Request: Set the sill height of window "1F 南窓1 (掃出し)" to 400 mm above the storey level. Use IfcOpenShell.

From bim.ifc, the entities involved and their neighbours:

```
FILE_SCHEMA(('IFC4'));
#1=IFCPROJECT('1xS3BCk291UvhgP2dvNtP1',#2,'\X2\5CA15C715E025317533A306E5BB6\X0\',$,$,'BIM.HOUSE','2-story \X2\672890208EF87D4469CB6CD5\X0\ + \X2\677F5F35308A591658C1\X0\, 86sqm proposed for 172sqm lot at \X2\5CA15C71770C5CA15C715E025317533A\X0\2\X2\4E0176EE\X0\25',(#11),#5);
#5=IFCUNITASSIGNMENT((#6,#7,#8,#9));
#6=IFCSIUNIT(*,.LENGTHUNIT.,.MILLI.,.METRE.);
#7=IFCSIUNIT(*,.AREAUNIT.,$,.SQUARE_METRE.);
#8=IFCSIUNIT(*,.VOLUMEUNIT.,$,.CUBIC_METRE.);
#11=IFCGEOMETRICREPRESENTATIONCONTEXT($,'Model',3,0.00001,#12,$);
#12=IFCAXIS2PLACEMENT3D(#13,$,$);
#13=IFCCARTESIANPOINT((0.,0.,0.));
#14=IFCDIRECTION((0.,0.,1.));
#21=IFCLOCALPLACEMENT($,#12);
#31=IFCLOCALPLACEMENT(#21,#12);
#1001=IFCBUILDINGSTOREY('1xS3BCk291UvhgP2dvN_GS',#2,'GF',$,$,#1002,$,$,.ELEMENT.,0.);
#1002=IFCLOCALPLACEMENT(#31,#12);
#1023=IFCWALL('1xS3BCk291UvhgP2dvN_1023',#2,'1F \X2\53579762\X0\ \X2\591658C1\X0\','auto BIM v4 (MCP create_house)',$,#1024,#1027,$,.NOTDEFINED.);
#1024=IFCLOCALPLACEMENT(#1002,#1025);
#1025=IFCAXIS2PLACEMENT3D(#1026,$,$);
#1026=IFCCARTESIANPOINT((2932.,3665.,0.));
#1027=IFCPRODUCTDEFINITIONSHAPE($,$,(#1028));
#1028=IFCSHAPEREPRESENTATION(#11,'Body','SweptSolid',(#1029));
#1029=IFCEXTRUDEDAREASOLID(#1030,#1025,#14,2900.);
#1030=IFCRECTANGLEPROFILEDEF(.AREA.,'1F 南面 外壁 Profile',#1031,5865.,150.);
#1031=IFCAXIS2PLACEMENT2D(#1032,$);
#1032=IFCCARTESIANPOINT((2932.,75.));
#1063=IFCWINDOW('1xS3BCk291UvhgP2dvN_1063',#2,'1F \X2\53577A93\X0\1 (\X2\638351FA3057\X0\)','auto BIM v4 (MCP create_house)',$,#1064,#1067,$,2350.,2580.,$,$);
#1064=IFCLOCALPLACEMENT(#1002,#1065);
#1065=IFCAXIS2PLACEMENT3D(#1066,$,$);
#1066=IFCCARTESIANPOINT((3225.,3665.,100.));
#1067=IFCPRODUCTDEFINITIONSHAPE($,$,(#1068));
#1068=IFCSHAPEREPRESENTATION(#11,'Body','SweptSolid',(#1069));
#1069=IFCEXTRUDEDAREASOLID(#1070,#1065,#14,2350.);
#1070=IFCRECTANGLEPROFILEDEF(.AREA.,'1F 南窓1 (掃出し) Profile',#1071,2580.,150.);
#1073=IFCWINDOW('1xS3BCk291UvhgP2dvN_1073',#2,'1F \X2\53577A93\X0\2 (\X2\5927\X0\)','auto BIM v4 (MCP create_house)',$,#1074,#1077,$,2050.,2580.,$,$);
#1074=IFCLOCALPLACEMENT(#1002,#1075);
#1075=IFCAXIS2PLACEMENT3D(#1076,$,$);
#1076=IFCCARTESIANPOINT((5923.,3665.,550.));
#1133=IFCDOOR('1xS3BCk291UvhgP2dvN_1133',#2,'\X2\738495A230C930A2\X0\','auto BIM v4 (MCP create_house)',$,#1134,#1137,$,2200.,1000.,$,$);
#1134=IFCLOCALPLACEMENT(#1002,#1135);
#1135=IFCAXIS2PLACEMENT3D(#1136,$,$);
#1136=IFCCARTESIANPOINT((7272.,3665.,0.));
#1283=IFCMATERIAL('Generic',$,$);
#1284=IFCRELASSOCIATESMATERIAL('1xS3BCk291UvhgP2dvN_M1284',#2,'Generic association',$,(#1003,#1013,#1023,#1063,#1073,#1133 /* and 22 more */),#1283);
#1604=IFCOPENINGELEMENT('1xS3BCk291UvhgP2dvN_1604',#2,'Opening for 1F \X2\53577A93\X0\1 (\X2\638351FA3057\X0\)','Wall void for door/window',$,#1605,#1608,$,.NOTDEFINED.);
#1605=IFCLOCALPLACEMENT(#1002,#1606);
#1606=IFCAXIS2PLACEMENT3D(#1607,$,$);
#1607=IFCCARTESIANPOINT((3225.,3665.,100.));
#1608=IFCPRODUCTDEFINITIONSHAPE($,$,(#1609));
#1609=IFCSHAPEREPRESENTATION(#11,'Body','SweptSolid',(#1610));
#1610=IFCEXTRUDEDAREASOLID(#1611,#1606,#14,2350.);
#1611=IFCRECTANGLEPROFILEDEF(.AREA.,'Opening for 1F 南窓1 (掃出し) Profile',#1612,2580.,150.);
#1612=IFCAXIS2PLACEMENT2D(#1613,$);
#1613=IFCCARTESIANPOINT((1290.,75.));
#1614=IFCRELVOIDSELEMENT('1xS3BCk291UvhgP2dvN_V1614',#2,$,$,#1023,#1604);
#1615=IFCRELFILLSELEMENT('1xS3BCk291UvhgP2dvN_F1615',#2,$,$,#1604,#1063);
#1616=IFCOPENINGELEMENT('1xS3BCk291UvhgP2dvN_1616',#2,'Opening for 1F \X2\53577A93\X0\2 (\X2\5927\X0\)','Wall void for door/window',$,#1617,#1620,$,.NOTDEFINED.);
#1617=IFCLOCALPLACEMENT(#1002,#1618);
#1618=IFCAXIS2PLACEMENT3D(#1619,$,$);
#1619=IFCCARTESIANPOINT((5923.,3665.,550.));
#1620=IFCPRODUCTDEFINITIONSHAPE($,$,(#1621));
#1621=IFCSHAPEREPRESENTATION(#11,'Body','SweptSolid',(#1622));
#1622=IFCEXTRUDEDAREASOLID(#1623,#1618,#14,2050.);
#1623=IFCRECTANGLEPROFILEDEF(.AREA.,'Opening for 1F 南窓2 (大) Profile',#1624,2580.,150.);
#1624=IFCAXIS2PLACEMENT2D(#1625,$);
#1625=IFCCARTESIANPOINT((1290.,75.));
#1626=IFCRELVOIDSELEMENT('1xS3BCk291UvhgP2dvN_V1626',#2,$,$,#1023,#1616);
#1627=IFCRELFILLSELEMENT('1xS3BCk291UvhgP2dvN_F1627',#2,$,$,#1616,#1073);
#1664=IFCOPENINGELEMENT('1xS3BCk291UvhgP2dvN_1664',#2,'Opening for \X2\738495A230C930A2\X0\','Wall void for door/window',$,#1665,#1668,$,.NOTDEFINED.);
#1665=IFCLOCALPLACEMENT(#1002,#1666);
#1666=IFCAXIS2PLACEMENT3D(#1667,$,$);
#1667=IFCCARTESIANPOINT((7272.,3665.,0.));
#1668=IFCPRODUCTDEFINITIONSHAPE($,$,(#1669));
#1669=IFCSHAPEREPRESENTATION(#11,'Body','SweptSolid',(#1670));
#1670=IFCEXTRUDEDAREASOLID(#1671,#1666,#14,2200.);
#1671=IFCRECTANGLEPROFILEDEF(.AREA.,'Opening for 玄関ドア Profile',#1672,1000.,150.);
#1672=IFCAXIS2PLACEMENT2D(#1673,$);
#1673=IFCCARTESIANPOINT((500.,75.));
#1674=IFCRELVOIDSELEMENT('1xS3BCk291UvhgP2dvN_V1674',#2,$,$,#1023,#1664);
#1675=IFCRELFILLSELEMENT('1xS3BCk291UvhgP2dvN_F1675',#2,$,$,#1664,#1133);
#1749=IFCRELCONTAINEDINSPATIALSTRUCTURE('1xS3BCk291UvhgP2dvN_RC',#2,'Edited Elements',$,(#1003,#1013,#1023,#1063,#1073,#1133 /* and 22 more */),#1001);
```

```python
import numpy as np
import ifcopenshell
import ifcopenshell.api.geometry
import ifcopenshell.geom
import ifcopenshell.util.element
import ifcopenshell.util.placement
import ifcopenshell.util.shape
import ifcopenshell.util.unit

model = ifcopenshell.open("bim.ifc")
unit_scale = ifcopenshell.util.unit.calculate_unit_scale(model)

window = model.by_guid("1xS3BCk291UvhgP2dvN_1063")
opening = window.FillsVoids[0].RelatingOpeningElement
storey = ifcopenshell.util.element.get_container(window, ifc_class="IfcBuildingStorey")
level = ifcopenshell.util.placement.get_local_placement(storey.ObjectPlacement)[2, 3]

# The opening's origin need not be at the sill, so measure its lowest point.
shape = ifcopenshell.geom.create_shape(ifcopenshell.geom.settings(), opening)
bottom = ifcopenshell.util.shape.get_shape_bottom_elevation(shape, shape.geometry) / unit_scale
dz = level + 0.4 / unit_scale - bottom

shift = np.array([0.0, 0.0, dz])
# The window is not placed relative to its opening, so move both.
for product in (opening, window):
    matrix = ifcopenshell.util.placement.get_local_placement(product.ObjectPlacement)
    matrix[:3, 3] += shift
    ifcopenshell.api.geometry.edit_object_placement(model, product=product, matrix=matrix, is_si=False)

print(f"moved by {dz * unit_scale:+.3f} m")

model.write("bim_edited.ifc")
```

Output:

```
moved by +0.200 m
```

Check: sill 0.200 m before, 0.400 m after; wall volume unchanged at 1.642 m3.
